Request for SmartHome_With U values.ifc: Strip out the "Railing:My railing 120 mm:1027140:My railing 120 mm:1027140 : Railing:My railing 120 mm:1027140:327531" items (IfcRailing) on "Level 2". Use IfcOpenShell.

First a look at what the model holds.

```python
import ifcopenshell
import ifcopenshell.util.element

model = ifcopenshell.open("SmartHome_With U values.ifc")
print(model.schema)
storey = next(s for s in model.by_type("IfcBuildingStorey") if s.Name == "Level 2")
railings = [e for e in ifcopenshell.util.element.get_decomposition(storey) if e.is_a("IfcRailing")]
seen = {}
for e in railings:
    element_type = ifcopenshell.util.element.get_type(e)
    name = element_type.Name if element_type not in (None, e) else None
    seen[name] = seen.get(name, 0) + 1
for name, count in sorted(seen.items(), key=str):
    print(count, "x", name)
```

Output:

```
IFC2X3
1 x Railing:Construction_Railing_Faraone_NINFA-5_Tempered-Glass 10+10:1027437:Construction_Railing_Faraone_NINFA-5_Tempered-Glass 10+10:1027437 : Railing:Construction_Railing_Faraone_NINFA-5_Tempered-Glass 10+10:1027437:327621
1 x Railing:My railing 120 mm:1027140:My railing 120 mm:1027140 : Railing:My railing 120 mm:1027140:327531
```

```python
import ifcopenshell
import ifcopenshell.api.root
import ifcopenshell.util.element

model = ifcopenshell.open("SmartHome_With U values.ifc")

storey = next(s for s in model.by_type("IfcBuildingStorey") if s.Name == "Level 2")
railings = [e for e in ifcopenshell.util.element.get_decomposition(storey) if e.is_a("IfcRailing")]
targets = [e for e in railings if (t := ifcopenshell.util.element.get_type(e)) not in (None, e) and t.Name == "Railing:My railing 120 mm:1027140:My railing 120 mm:1027140 : Railing:My railing 120 mm:1027140:327531"]

for e in targets:
    ifcopenshell.api.root.remove_product(model, product=e)
print(len(targets), "removed")

model.write("SmartHome_With U values_edited.ifc")
```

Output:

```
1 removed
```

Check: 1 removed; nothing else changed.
